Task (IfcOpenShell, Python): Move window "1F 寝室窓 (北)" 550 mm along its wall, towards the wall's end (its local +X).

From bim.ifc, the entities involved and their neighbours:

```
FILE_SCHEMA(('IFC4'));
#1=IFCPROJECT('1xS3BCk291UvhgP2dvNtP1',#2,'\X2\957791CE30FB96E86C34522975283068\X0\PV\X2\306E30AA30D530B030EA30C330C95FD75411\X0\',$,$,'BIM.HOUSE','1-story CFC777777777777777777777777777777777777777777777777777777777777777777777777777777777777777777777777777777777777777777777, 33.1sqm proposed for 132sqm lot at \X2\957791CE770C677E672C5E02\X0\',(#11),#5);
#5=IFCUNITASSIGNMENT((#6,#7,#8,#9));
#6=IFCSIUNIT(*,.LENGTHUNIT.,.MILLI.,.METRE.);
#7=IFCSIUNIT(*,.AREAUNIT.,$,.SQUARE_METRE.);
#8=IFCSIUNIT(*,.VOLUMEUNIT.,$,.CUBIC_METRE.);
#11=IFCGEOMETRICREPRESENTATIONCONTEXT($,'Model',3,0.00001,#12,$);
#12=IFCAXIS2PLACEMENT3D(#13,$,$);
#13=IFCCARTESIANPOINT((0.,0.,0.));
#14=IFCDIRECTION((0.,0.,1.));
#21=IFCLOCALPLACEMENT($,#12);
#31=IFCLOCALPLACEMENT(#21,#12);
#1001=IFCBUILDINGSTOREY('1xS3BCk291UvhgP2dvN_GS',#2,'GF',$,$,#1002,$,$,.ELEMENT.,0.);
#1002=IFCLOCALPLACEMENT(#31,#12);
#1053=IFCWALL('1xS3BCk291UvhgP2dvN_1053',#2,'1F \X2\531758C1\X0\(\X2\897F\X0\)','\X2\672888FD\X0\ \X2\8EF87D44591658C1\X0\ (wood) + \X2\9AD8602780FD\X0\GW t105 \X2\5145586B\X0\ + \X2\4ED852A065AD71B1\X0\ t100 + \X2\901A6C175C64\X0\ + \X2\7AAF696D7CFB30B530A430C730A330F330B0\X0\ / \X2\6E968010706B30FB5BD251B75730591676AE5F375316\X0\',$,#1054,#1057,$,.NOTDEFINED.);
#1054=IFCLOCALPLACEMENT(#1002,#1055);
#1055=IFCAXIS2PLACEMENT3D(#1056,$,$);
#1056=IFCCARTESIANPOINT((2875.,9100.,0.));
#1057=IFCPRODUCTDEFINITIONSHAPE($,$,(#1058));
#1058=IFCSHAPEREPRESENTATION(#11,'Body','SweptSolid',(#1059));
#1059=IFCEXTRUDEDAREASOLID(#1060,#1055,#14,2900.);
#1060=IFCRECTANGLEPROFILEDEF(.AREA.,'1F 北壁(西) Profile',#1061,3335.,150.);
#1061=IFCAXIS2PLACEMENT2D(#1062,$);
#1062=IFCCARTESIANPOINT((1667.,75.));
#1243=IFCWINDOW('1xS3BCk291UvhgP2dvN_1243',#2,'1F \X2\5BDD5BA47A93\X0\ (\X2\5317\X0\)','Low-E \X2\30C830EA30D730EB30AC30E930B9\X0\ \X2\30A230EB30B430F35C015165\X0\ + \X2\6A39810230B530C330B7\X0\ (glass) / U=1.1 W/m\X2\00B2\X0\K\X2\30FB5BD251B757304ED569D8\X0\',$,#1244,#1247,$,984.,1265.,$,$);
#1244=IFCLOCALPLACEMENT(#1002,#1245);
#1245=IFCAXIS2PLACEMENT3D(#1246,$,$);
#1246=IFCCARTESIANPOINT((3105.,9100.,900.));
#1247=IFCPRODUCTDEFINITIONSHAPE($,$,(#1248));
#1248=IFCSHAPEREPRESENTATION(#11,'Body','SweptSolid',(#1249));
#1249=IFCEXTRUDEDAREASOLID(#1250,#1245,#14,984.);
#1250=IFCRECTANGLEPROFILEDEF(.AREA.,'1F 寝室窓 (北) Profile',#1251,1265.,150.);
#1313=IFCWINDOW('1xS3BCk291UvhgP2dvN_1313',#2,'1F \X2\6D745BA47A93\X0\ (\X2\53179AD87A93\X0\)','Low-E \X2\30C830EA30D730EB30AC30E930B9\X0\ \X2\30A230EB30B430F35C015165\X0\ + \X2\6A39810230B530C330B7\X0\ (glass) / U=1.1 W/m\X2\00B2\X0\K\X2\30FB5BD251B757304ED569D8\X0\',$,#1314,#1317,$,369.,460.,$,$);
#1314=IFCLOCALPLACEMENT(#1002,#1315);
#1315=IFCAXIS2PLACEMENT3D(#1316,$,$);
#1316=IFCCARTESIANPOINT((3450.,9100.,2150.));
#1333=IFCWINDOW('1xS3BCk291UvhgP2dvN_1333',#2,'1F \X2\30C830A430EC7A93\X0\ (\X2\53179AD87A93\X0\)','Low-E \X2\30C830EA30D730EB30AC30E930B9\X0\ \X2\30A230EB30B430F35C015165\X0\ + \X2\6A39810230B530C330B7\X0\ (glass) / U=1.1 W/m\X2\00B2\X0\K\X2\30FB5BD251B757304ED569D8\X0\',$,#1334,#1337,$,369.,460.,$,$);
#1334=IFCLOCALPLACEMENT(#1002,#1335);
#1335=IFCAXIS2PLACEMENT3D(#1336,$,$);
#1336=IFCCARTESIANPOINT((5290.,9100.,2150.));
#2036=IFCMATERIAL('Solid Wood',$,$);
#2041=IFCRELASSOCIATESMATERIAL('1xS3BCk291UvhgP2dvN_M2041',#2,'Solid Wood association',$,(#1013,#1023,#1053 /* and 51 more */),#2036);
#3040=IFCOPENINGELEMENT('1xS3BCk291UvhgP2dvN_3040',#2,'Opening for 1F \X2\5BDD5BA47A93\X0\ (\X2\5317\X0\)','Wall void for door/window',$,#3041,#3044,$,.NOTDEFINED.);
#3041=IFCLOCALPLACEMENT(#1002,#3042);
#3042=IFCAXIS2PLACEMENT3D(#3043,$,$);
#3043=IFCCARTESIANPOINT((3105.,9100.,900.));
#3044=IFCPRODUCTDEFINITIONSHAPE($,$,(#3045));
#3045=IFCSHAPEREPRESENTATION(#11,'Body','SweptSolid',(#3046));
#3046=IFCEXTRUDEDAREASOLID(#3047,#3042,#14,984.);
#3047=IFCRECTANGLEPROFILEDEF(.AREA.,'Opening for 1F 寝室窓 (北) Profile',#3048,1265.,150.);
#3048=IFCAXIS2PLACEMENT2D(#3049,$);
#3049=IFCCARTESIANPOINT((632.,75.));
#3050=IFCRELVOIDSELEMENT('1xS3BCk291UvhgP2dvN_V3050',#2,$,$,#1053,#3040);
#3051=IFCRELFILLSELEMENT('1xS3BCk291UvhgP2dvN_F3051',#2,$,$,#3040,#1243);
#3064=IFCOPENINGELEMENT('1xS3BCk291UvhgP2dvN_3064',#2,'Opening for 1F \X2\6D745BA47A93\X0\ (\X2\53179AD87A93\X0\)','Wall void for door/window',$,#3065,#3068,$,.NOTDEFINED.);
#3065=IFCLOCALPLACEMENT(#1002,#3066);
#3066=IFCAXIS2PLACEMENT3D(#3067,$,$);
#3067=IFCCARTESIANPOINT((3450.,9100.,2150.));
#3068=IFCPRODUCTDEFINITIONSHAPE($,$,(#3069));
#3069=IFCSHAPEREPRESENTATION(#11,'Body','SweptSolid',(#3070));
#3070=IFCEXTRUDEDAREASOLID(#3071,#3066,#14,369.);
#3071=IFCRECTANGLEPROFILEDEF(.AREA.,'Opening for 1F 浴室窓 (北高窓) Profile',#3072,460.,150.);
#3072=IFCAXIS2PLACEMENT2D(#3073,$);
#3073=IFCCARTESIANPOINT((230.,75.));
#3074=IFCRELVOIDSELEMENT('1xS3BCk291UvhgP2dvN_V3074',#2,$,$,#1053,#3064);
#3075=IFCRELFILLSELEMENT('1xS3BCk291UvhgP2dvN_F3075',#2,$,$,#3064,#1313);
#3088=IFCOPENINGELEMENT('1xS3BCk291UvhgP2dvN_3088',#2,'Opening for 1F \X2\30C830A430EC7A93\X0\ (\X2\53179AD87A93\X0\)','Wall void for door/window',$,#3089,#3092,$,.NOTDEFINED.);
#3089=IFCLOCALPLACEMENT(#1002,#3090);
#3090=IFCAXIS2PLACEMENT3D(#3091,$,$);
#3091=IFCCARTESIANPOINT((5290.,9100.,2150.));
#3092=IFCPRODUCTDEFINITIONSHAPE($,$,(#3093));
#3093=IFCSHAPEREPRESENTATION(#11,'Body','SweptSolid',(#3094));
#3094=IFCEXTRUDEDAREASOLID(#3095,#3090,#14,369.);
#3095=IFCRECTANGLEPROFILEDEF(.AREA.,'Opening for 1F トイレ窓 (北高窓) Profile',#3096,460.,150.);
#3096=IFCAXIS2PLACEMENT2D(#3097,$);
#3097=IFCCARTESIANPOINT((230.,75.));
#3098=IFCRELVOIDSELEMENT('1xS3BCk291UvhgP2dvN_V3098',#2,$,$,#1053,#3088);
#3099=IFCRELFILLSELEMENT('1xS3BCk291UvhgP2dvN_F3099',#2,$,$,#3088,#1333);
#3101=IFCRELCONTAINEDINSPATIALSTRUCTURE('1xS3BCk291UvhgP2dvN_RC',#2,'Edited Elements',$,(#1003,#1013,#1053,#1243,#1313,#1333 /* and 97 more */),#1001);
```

```python
import ifcopenshell
import ifcopenshell.api.geometry
import ifcopenshell.util.placement

model = ifcopenshell.open("bim.ifc")

window = model.by_id(1243)
opening = window.FillsVoids[0].RelatingOpeningElement
wall = opening.VoidsElements[0].RelatingBuildingElement

wall_matrix = ifcopenshell.util.placement.get_local_placement(wall.ObjectPlacement)
shift = wall_matrix[:3, 0] * 550.0
before = ifcopenshell.util.placement.get_local_placement(window.ObjectPlacement)[:3, 3].copy()

# The window is not placed relative to its opening, so move both.
for product in (opening, window):
    matrix = ifcopenshell.util.placement.get_local_placement(product.ObjectPlacement)
    matrix[:3, 3] += shift
    ifcopenshell.api.geometry.edit_object_placement(model, product=product, matrix=matrix, is_si=False)

after = ifcopenshell.util.placement.get_local_placement(window.ObjectPlacement)[:3, 3]
print("window moved by", (after - before).round(3) + 0.0)

model.write("bim_rev.ifc")
```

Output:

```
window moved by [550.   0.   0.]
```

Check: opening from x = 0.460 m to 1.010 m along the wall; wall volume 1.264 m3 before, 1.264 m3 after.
